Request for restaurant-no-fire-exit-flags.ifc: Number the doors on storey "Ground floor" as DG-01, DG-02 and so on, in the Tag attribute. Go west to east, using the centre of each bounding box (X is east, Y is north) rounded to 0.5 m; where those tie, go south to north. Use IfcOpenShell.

First a look at what the model holds.

```python
import ifcopenshell
import ifcopenshell.util.element
import ifcopenshell.util.placement

model = ifcopenshell.open("restaurant-no-fire-exit-flags.ifc")
print(model.schema)
storey = next(s for s in model.by_type("IfcBuildingStorey") if s.Name == "Ground floor")
doors = [e for e in ifcopenshell.util.element.get_decomposition(storey) if e.is_a("IfcDoor")]
for e in sorted(doors, key=lambda e: e.id()):
    origin = ifcopenshell.util.placement.get_local_placement(e.ObjectPlacement)[:3, 3]
    print(e.id(), e.Tag, e.Name, origin.round(2) + 0.0, sep=" | ")
```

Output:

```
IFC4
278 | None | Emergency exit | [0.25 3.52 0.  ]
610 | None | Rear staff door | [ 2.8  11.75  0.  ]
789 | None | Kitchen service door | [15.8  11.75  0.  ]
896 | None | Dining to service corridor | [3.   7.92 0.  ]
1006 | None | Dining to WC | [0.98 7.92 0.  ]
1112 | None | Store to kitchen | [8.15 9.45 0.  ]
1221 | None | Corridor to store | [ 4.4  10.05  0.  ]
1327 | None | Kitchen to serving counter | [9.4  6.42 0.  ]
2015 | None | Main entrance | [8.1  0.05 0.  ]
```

```python
import ifcopenshell
import ifcopenshell.geom
import ifcopenshell.util.element
import ifcopenshell.util.shape

model = ifcopenshell.open("restaurant-no-fire-exit-flags.ifc")
settings = ifcopenshell.geom.settings()
settings.set("use-world-coords", True)


def centre(element):
    shape = ifcopenshell.geom.create_shape(settings, element)
    return ifcopenshell.util.shape.get_bbox_centroid(shape.geometry)


storey = next(s for s in model.by_type("IfcBuildingStorey") if s.Name == "Ground floor")
doors = [e for e in ifcopenshell.util.element.get_decomposition(storey) if e.is_a("IfcDoor")]

# Insertion points can sit at a corner or the storey origin, so sort by the geometry (in metres).
centres = {e: centre(e) for e in doors}
doors.sort(key=lambda e: (round(centres[e][0] / 0.5), centres[e][1]))

for i, e in enumerate(doors, start=1):
    number = f"DG-{i:02d}"
    e.Tag = number
    print(e.id(), number)

model.write("restaurant-no-fire-exit-flags_v2.ifc")
```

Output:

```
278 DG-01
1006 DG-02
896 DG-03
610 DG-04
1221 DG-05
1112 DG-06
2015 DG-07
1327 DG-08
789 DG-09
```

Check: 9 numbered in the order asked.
